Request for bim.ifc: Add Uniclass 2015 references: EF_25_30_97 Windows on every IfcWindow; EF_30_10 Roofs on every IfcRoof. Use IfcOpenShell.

First a look at what the model holds.

```python
import ifcopenshell

model = ifcopenshell.open("bim.ifc")
print(model.schema)
print("classifications:", [c.Name for c in model.by_type("IfcClassification")])
for ifc_class in ("IfcDoor", "IfcRoof", "IfcStair", "IfcWall", "IfcWindow"):
    print(ifc_class, len(model.by_type(ifc_class)))
```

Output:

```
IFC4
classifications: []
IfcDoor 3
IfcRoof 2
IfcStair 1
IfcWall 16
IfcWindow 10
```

```python
import ifcopenshell
import ifcopenshell.api.classification

model = ifcopenshell.open("bim.ifc")

system = ifcopenshell.api.classification.add_classification(model, classification="Uniclass 2015")

codes = {
    "IfcWindow": ("EF_25_30_97", "Windows"),
    "IfcRoof": ("EF_30_10", "Roofs"),
}
for ifc_class, (code, name) in codes.items():
    products = model.by_type(ifc_class)
    ifcopenshell.api.classification.add_reference(
        model, products=products, classification=system, identification=code, name=name
    )
    print(code, len(products))

model.write("bim_v2.ifc")
```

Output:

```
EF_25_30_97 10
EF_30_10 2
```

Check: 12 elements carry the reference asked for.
